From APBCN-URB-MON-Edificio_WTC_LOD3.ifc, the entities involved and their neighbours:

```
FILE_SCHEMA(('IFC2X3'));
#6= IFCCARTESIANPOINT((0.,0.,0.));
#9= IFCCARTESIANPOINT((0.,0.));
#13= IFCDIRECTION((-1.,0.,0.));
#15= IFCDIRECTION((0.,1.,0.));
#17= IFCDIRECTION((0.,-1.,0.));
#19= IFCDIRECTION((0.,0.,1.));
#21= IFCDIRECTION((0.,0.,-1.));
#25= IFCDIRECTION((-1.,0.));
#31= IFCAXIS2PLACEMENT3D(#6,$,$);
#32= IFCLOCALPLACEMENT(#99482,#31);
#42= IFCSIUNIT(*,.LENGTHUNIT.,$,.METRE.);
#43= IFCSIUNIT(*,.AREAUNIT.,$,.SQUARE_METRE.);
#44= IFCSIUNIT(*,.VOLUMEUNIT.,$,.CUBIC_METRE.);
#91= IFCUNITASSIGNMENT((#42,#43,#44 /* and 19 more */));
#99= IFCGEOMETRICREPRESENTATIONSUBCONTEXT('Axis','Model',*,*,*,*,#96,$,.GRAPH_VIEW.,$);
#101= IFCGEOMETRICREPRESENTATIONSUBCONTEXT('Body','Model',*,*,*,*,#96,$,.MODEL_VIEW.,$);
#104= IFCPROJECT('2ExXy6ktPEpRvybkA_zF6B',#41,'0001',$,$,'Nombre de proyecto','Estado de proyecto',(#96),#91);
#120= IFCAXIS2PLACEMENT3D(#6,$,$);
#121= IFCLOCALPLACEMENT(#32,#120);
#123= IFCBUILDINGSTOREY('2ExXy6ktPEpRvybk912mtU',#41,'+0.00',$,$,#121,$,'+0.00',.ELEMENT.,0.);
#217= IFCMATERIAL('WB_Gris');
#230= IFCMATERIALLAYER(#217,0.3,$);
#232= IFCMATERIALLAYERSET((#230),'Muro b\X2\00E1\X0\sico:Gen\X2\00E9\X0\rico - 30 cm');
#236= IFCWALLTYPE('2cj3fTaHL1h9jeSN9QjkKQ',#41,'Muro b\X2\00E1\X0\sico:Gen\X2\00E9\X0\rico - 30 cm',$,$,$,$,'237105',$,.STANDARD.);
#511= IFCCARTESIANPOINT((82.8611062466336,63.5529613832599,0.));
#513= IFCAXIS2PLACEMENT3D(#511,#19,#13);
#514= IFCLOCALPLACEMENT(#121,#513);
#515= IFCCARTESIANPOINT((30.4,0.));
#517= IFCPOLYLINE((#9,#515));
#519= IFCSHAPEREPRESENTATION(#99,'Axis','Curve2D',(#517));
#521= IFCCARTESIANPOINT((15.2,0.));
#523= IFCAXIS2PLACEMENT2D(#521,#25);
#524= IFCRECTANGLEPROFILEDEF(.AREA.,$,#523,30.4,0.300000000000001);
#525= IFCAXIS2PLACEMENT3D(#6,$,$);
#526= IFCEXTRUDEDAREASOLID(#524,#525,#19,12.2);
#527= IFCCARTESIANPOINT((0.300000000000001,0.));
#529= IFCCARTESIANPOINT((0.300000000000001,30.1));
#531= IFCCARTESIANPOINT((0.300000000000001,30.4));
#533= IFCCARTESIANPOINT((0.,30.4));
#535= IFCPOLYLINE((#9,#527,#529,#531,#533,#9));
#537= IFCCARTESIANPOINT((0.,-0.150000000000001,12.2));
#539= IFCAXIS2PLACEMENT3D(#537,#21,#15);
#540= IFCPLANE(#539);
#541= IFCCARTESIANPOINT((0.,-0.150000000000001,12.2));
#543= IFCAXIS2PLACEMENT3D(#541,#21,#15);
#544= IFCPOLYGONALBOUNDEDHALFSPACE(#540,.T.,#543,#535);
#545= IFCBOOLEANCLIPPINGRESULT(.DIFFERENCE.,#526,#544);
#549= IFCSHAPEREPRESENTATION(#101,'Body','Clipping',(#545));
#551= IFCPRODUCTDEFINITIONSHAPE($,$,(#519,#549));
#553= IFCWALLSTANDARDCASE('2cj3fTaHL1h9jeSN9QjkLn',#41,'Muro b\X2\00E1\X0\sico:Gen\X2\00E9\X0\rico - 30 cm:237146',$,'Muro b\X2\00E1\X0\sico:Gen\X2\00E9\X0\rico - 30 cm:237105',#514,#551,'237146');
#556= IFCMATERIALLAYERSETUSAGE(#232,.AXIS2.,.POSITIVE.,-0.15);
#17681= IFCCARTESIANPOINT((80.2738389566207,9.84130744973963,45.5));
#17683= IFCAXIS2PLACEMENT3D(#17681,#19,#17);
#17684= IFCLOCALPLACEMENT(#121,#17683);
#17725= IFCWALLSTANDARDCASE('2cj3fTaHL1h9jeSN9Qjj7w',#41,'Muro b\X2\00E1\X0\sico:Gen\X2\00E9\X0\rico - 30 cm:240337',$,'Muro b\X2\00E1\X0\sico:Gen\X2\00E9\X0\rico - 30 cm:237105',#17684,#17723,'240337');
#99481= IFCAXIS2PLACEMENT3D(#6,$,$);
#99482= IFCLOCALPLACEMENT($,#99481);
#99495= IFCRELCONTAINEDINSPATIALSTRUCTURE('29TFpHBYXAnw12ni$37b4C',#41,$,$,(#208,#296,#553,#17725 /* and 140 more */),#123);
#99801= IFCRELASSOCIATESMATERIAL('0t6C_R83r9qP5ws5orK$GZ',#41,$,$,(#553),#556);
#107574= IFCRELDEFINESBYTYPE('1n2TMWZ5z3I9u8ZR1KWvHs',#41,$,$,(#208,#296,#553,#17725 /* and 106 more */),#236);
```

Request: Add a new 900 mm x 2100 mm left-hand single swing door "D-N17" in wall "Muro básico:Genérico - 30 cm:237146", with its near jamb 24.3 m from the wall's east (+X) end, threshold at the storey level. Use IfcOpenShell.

```python
import numpy as np
import ifcopenshell
import ifcopenshell.api.feature
import ifcopenshell.api.geometry
import ifcopenshell.api.root
import ifcopenshell.api.spatial
import ifcopenshell.api.type
import ifcopenshell.geom
import ifcopenshell.util.element
import ifcopenshell.util.placement
import ifcopenshell.util.representation
import ifcopenshell.util.shape
import ifcopenshell.util.unit

model = ifcopenshell.open("APBCN-URB-MON-Edificio_WTC_LOD3.ifc")
unit_scale = ifcopenshell.util.unit.calculate_unit_scale(model)
settings = ifcopenshell.geom.settings()


def volume(element):
    """Net volume in cubic metres, openings subtracted."""
    shape = ifcopenshell.geom.create_shape(settings, element)
    return ifcopenshell.util.shape.get_volume(shape.geometry)


wall = model.by_guid("2cj3fTaHL1h9jeSN9QjkLn")
storey = ifcopenshell.util.element.get_container(wall, ifc_class="IfcBuildingStorey")
context = ifcopenshell.util.representation.get_context(model, "Model", "Body", "MODEL_VIEW")
before = volume(wall)

width, height, from_end, sill = 0.9, 2.1, 24.3, 0.0  # metres

# The wall runs along its own X axis, and the end named is its -X end.
wall_shape = ifcopenshell.geom.create_shape(settings, wall)
x, y, z = ifcopenshell.util.shape.get_vertices(wall_shape.geometry).T
start = x.min() + from_end
face, thickness = float(y.min()), float(y.max() - y.min())
wall_matrix = ifcopenshell.util.placement.get_local_placement(wall.ObjectPlacement)
level = ifcopenshell.util.placement.get_local_placement(storey.ObjectPlacement)[2, 3]


def in_wall(x, y):
    """Placement at x, y metres in the wall's axes, at sill height."""
    matrix = wall_matrix.copy()
    matrix[:, 3] = wall_matrix @ np.array([x / unit_scale, y / unit_scale, 0.0, 1.0])
    matrix[2, 3] = level + sill / unit_scale
    return matrix


# Opening: a box that overshoots both wall faces by 50 mm.
opening = ifcopenshell.api.root.create_entity(model, ifc_class="IfcOpeningElement")
box = ifcopenshell.api.geometry.add_wall_representation(
    model, context=context, length=width, height=height, thickness=thickness + 0.1
)
ifcopenshell.api.geometry.assign_representation(model, product=opening, representation=box)
ifcopenshell.api.geometry.edit_object_placement(model, product=opening, matrix=in_wall(start, face - 0.05), is_si=False)
ifcopenshell.api.feature.add_feature(model, feature=opening, element=wall)

door = ifcopenshell.api.root.create_entity(model, ifc_class="IfcDoor", name="D-N17")
door.OverallWidth, door.OverallHeight = width / unit_scale, height / unit_scale
body = ifcopenshell.api.geometry.add_door_representation(
    model,
    context=context,
    overall_width=door.OverallWidth,
    overall_height=door.OverallHeight,
    operation_type="SINGLE_SWING_LEFT",
    lining_properties={"LiningDepth": thickness / unit_scale, "ThresholdDepth": thickness / unit_scale},
)
ifcopenshell.api.geometry.assign_representation(model, product=door, representation=body)
ifcopenshell.api.spatial.assign_container(model, products=[door], relating_structure=storey)
fills = ifcopenshell.api.feature.add_filling(model, opening=opening, element=door)
fills.OwnerHistory = door.OwnerHistory  # required in IFC2X3

# IFC2X3 keeps the operation on the door style.
style = ifcopenshell.api.root.create_entity(model, ifc_class="IfcDoorStyle", name="D-N17")
style.OperationType, style.ConstructionType = "SINGLE_SWING_LEFT", "NOTDEFINED"
style.ParameterTakesPrecedence = style.Sizeable = False
ifcopenshell.api.type.assign_type(model, related_objects=[door], relating_type=style)

# The lining spans the wall, so the door starts at the wall face.
ifcopenshell.api.geometry.edit_object_placement(model, product=door, matrix=in_wall(start, face), is_si=False)

after = volume(wall)

print(f"wall volume {before:.3f} -> {after:.3f} m3")

model.write("APBCN-URB-MON-Edificio_WTC_LOD3_v2.ifc")
```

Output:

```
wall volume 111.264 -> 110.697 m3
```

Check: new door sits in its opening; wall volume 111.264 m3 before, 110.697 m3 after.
